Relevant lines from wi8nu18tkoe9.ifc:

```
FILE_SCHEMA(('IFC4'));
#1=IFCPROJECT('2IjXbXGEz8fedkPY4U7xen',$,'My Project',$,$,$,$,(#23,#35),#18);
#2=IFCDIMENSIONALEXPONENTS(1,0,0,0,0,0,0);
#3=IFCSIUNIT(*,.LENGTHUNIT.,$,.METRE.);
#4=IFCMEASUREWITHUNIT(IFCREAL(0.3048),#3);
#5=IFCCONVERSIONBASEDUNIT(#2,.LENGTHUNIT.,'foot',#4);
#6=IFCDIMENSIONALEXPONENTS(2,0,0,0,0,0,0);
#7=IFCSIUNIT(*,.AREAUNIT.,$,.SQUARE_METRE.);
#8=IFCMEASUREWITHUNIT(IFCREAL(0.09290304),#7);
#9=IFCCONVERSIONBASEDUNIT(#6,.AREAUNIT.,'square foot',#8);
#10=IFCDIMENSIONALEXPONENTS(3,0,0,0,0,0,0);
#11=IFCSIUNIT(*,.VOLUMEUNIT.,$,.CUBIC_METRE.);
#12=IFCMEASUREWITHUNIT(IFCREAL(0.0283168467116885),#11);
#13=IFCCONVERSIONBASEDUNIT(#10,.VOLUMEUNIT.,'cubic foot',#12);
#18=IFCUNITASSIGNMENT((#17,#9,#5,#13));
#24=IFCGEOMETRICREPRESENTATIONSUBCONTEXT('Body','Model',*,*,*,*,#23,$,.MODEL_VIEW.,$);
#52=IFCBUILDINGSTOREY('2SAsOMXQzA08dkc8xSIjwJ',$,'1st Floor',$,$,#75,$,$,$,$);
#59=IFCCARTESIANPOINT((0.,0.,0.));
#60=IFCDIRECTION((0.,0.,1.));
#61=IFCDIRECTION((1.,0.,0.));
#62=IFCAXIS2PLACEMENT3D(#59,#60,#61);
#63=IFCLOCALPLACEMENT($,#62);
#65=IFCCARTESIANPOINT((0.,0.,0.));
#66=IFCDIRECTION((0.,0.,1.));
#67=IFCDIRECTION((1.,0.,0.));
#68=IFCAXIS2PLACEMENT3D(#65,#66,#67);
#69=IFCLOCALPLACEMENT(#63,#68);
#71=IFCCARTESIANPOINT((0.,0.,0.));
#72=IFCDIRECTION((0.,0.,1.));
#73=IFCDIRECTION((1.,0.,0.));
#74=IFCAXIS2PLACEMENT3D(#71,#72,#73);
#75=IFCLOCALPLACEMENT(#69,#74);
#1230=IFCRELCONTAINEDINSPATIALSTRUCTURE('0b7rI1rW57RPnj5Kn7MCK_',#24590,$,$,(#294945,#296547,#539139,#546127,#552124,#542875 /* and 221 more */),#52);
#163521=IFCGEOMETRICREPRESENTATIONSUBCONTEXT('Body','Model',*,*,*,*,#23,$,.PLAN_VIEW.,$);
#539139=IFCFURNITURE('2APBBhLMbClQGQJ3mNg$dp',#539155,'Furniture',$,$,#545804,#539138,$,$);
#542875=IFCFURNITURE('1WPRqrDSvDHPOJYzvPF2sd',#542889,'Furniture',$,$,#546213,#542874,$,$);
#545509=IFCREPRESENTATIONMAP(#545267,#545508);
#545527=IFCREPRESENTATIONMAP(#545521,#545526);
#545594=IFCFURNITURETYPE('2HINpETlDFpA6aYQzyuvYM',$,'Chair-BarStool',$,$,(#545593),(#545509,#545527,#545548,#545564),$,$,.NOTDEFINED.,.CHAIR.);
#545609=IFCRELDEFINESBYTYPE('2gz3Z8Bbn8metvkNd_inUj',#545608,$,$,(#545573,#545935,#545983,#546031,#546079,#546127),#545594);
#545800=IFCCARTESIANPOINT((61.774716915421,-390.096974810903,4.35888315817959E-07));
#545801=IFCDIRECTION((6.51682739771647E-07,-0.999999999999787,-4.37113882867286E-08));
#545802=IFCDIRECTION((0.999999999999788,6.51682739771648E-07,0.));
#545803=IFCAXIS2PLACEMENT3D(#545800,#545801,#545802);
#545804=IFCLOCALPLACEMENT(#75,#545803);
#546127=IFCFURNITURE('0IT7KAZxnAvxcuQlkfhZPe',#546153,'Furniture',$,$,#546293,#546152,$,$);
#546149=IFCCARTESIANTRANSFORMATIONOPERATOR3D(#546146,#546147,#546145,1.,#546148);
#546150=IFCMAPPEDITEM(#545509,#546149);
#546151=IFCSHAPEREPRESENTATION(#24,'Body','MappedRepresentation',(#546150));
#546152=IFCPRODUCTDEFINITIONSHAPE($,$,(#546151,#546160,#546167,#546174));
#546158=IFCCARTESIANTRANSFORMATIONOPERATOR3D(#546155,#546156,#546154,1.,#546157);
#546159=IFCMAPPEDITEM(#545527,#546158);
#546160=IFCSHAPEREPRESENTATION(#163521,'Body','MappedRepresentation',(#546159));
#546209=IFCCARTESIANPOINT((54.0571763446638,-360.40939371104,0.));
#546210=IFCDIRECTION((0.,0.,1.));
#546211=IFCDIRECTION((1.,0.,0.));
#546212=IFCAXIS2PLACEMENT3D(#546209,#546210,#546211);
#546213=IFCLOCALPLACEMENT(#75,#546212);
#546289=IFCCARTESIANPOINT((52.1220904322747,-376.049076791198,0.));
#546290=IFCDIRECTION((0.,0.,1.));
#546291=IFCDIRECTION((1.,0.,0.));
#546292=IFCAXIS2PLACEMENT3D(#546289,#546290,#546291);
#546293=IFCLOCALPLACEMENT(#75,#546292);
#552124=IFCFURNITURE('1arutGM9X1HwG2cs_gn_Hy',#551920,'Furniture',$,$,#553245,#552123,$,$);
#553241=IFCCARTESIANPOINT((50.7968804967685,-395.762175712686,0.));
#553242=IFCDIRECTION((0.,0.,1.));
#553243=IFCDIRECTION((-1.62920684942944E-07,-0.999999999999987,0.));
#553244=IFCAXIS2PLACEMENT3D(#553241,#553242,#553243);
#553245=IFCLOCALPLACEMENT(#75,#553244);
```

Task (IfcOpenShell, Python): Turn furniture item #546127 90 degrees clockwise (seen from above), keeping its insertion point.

```python
import ifcopenshell
import ifcopenshell.api.geometry
import ifcopenshell.util.placement

model = ifcopenshell.open("wi8nu18tkoe9.ifc")

item = model.by_guid("0IT7KAZxnAvxcuQlkfhZPe")
matrix = ifcopenshell.util.placement.get_local_placement(item.ObjectPlacement)
matrix = matrix @ ifcopenshell.util.placement.rotation(-90, "Z")
ifcopenshell.api.geometry.edit_object_placement(model, product=item, matrix=matrix, is_si=False)

print(ifcopenshell.util.placement.get_local_placement(item.ObjectPlacement).round(3) + 0.0)

model.write("wi8nu18tkoe9_v2.ifc")
```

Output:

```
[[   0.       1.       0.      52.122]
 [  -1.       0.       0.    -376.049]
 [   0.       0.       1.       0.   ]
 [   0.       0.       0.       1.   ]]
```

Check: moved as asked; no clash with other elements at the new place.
